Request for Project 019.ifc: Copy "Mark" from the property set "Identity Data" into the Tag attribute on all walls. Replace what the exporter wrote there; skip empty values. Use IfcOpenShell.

First a look at what the model holds.

```python
import ifcopenshell
import ifcopenshell.util.element

model = ifcopenshell.open("Project 019.ifc")
print(model.schema)
walls = model.by_type("IfcWall")
print(len(walls), "walls")
for e in walls[:8]:
    source = ifcopenshell.util.element.get_pset(e, "Identity Data", "Mark")
    target = e.Tag
    print(e.id(), repr(source), repr(target), sep=" | ")
```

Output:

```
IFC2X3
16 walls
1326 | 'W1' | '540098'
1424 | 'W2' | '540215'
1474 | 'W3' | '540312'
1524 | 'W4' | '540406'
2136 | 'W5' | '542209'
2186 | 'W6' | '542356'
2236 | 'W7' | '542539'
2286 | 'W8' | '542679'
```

```python
import ifcopenshell
import ifcopenshell.util.element

model = ifcopenshell.open("Project 019.ifc")

count = 0
for e in model.by_type("IfcWall"):
    value = ifcopenshell.util.element.get_pset(e, "Identity Data", "Mark")
    current = e.Tag
    if not value or not value.strip() or current == value:
        continue
    e.Tag = value
    count += 1

print(count, "walls updated")

model.write("Project 019_updated.ifc")
```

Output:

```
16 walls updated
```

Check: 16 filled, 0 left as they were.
